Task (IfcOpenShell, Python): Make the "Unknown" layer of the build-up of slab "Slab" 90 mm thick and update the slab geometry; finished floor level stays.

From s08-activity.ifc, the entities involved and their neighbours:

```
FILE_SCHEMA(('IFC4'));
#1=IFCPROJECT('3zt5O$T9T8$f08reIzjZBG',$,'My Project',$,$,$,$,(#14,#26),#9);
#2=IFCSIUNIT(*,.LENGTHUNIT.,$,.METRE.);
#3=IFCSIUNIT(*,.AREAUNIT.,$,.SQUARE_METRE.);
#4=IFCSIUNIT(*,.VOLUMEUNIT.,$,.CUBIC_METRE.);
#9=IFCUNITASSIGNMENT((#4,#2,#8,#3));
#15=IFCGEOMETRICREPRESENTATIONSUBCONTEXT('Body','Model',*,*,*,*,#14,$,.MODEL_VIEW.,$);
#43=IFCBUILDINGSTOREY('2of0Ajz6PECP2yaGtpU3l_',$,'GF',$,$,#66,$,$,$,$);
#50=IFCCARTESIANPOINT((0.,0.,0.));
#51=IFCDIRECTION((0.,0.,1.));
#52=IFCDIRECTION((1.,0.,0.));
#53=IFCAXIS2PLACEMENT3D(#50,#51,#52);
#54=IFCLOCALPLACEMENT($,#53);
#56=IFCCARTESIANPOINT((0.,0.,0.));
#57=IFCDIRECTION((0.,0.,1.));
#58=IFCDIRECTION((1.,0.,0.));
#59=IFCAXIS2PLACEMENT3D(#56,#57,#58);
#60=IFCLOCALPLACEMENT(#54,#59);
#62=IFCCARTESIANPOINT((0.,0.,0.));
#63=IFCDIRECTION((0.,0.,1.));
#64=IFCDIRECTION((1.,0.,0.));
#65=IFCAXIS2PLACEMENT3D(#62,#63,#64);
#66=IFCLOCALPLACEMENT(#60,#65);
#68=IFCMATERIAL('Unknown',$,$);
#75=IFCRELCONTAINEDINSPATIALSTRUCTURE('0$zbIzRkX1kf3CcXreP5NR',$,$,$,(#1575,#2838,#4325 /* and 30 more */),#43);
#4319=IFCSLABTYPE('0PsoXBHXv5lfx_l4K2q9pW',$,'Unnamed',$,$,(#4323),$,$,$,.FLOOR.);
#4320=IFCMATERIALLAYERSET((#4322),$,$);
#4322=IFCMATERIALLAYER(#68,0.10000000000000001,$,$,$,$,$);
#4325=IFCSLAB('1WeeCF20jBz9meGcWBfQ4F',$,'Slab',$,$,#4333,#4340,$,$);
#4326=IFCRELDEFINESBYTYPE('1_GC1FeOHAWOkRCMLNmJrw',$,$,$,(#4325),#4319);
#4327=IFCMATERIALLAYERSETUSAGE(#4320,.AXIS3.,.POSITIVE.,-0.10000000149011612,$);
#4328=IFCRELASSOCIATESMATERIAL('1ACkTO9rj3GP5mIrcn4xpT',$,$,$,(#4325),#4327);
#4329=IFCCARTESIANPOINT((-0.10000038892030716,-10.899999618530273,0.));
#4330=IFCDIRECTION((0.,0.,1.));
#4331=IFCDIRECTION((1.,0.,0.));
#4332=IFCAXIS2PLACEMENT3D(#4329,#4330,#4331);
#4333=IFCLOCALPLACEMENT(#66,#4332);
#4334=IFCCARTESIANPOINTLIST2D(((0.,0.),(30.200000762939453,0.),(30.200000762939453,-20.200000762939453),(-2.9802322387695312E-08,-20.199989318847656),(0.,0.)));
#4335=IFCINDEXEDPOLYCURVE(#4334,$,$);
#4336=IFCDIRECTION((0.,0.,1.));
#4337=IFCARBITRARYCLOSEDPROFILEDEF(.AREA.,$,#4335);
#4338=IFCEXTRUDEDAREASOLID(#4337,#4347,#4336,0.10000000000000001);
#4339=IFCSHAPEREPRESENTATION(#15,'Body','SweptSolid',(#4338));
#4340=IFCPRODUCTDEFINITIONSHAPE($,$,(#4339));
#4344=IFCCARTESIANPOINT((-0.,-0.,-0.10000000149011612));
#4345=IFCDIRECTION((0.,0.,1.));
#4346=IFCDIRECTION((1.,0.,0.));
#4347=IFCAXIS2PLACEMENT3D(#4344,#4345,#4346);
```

```python
import ifcopenshell
import ifcopenshell.util.element
import ifcopenshell.util.representation
import ifcopenshell.util.unit

model = ifcopenshell.open("s08-activity.ifc")
unit_scale = ifcopenshell.util.unit.calculate_unit_scale(model)

layer_set = model.by_id(4320)
layer = next(l for l in layer_set.MaterialLayers if l.Material and l.Material.Name == "Unknown")
change = 0.09 / unit_scale - layer.LayerThickness
layer.LayerThickness += change

# Geometry does not follow the layer set by itself.
slabs = [e for e in ifcopenshell.util.element.get_elements_by_material(model, layer_set) if e.is_a("IfcSlab")]
for slab in sorted(slabs, key=lambda e: e.id()):
    body = ifcopenshell.util.representation.get_representation(slab, "Model", "Body")
    solid = body.Items[0]
    old_depth = solid.Depth
    solid.Depth += change
    # Extruded upwards: lower the start of the extrusion so the top stays.
    x, y, z = solid.Position.Location.Coordinates
    solid.Position.Location = model.createIfcCartesianPoint((x, y, z - change))
    print(slab.id(), f"{old_depth:g} -> {solid.Depth:g}")

# The layers are counted up from the underside, which has moved.
for usage in {ifcopenshell.util.element.get_material(slab) for slab in slabs}:
    usage.OffsetFromReferenceLine -= change

model.write("s08-activity_edited.ifc")
```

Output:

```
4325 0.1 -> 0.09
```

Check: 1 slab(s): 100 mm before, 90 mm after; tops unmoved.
